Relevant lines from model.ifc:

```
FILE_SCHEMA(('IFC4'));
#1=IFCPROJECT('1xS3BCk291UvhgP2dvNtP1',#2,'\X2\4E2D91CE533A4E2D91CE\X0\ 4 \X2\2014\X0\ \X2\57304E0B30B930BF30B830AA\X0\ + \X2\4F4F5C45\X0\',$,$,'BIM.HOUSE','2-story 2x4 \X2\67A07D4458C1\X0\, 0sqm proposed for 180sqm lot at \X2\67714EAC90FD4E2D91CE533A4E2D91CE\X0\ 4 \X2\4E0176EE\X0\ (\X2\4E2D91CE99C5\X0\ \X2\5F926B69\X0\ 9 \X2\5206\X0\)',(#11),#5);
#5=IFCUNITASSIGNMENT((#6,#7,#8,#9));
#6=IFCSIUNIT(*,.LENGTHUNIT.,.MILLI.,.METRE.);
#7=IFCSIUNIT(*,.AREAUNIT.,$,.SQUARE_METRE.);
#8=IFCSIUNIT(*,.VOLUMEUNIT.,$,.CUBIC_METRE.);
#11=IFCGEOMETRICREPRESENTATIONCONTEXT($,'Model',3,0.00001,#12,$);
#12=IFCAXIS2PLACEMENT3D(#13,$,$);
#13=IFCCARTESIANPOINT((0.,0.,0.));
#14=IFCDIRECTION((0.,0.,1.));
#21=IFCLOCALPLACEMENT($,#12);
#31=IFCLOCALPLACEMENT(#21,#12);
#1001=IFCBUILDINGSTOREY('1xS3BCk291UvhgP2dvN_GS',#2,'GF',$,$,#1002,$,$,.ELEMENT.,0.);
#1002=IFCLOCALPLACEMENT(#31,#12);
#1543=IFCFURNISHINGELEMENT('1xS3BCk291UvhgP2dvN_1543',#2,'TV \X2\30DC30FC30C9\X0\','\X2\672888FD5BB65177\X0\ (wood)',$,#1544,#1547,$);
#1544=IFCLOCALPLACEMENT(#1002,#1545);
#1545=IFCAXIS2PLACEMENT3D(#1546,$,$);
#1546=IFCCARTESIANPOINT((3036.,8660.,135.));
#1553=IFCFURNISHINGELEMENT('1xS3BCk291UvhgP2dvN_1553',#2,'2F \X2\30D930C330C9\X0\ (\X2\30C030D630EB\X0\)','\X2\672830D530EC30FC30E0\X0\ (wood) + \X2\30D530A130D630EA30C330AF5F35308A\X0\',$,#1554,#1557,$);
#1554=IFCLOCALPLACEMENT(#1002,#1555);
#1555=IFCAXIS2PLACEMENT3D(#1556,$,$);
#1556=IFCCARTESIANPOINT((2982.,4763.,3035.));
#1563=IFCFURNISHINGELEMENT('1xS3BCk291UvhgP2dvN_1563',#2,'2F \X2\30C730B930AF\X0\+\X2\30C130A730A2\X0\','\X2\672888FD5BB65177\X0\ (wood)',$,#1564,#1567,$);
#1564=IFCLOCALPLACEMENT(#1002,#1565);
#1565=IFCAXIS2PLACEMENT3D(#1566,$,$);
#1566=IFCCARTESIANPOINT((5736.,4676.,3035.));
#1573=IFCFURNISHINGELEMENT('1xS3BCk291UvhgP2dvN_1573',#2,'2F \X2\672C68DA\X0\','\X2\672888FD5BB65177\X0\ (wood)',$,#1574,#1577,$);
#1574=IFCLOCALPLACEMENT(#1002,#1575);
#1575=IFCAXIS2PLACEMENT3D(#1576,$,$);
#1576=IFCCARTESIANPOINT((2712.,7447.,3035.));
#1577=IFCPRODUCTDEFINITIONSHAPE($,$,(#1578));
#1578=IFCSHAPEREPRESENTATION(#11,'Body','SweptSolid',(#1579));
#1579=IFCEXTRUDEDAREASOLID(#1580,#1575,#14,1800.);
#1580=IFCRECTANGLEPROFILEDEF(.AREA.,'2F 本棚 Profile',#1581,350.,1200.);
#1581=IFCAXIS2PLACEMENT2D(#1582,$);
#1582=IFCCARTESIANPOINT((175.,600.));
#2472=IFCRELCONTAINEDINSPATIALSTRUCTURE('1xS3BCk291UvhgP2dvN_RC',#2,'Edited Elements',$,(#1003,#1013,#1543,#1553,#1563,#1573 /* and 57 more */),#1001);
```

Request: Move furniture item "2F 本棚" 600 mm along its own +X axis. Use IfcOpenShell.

```python
import ifcopenshell
import ifcopenshell.api.geometry
import ifcopenshell.util.placement

model = ifcopenshell.open("model.ifc")

item = model.by_id(1573)
matrix = ifcopenshell.util.placement.get_local_placement(item.ObjectPlacement)
matrix[:3, 3] += matrix[:3, 0] * 600.0
ifcopenshell.api.geometry.edit_object_placement(model, product=item, matrix=matrix, is_si=False)

print(ifcopenshell.util.placement.get_local_placement(item.ObjectPlacement).round(3) + 0.0)

model.write("model_rev.ifc")
```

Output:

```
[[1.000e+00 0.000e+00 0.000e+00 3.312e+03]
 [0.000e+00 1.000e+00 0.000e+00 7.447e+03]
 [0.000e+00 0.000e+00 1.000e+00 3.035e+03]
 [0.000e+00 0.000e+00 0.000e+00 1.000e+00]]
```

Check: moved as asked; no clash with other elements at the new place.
